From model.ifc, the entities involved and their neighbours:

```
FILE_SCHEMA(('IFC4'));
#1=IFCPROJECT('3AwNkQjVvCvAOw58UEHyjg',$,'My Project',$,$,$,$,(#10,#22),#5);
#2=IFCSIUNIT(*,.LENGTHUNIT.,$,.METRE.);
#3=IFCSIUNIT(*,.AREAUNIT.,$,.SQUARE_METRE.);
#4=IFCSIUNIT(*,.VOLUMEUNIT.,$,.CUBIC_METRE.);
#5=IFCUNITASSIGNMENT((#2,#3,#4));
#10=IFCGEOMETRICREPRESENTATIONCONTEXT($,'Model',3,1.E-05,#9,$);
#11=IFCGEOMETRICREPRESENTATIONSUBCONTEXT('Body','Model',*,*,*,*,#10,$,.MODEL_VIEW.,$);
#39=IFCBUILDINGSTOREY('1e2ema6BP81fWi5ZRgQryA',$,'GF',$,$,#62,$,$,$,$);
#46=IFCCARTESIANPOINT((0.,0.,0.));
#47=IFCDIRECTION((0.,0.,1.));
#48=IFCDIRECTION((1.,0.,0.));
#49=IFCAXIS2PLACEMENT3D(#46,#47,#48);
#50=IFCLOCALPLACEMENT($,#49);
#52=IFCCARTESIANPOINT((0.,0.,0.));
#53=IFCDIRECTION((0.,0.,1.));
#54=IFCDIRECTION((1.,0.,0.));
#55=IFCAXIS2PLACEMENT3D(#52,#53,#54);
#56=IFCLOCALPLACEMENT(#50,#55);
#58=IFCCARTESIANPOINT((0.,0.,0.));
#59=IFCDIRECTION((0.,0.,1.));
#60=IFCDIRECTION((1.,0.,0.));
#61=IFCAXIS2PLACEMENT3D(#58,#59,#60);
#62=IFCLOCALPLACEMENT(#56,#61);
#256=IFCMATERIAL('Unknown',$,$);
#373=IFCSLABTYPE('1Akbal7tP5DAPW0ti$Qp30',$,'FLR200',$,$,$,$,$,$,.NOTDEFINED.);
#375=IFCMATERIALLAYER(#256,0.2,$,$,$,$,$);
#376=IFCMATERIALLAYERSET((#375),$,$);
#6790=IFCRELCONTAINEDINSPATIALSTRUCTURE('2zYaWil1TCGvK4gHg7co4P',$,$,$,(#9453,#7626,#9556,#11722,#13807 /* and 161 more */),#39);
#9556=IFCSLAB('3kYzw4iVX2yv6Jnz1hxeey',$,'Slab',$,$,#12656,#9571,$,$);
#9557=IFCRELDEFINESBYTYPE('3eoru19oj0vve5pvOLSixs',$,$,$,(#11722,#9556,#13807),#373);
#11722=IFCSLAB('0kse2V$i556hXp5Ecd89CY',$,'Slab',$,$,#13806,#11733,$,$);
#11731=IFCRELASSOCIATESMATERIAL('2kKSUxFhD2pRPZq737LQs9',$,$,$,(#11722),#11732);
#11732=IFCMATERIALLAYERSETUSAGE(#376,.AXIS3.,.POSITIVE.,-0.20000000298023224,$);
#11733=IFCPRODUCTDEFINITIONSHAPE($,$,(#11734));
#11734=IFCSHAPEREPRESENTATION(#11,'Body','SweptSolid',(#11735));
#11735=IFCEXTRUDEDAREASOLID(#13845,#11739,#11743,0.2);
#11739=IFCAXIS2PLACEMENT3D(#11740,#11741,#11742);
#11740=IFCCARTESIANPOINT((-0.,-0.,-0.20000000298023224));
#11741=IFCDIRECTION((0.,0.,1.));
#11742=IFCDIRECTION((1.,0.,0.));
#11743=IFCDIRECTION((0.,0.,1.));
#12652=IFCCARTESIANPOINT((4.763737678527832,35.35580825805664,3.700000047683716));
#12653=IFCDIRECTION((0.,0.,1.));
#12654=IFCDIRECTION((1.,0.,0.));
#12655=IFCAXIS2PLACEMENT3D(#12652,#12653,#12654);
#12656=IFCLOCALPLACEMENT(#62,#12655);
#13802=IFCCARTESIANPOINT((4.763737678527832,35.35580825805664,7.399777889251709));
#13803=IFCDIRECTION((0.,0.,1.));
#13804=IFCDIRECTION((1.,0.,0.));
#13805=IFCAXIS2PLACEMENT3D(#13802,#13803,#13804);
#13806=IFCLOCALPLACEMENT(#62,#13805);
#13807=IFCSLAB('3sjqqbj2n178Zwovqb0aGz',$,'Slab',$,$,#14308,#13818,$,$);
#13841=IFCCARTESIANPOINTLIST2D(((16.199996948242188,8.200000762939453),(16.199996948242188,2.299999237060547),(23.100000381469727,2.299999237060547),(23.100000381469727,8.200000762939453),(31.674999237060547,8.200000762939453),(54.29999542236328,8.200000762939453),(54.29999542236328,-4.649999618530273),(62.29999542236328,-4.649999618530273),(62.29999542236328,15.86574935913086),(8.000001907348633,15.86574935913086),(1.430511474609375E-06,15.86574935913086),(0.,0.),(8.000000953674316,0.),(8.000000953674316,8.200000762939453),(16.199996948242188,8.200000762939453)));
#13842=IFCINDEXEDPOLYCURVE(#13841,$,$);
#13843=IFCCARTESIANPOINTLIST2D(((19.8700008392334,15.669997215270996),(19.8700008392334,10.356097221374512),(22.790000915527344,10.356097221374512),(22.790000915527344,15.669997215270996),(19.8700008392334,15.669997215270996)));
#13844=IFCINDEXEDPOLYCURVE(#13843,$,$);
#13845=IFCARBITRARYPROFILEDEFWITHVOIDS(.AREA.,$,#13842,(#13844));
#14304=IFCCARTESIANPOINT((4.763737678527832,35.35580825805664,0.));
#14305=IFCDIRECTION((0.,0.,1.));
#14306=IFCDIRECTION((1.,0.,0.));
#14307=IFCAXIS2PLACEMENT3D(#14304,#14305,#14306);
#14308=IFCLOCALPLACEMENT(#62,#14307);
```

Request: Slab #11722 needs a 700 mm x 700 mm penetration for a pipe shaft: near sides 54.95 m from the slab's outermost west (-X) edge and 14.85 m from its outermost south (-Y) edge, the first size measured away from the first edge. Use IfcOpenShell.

```python
import numpy as np
import ifcopenshell
import ifcopenshell.api.feature
import ifcopenshell.api.geometry
import ifcopenshell.api.root
import ifcopenshell.geom
import ifcopenshell.util.placement
import ifcopenshell.util.representation
import ifcopenshell.util.shape
import ifcopenshell.util.unit

model = ifcopenshell.open("model.ifc")
unit_scale = ifcopenshell.util.unit.calculate_unit_scale(model)
settings = ifcopenshell.geom.settings()


def volume(element):
    """Net volume in cubic metres, openings subtracted."""
    shape = ifcopenshell.geom.create_shape(settings, element)
    return ifcopenshell.util.shape.get_volume(shape.geometry)


slab = model.by_guid("0kse2V$i556hXp5Ecd89CY")
before = volume(slab)

# Extent in the slab's own axes, in metres. The edges named are its -X and -Y sides.
slab_shape = ifcopenshell.geom.create_shape(settings, slab)
vertices = ifcopenshell.util.shape.get_vertices(slab_shape.geometry)
x_min, y_min, bottom = vertices.min(axis=0)
top = vertices[:, 2].max()

opening = ifcopenshell.api.root.create_entity(model, ifc_class="IfcOpeningElement", name="Pipe shaft opening", predefined_type="OPENING")
context = ifcopenshell.util.representation.get_context(model, "Model", "Body", "MODEL_VIEW")
width, depth = 0.7, 0.7
outline = [(0.0, 0.0), (width, 0.0), (width, depth), (0.0, depth), (0.0, 0.0)]
# Overshoot both faces by 50 mm so the cut is clean.
shape = ifcopenshell.api.geometry.add_slab_representation(
    model, context=context, depth=top - bottom + 0.1, polyline=outline
)
ifcopenshell.api.geometry.assign_representation(model, product=opening, representation=shape)

matrix = ifcopenshell.util.placement.get_local_placement(slab.ObjectPlacement)
matrix[:, 3] = matrix @ np.append(np.array([x_min + 54.95, y_min + 14.85, bottom - 0.05]) / unit_scale, 1.0)
ifcopenshell.api.geometry.edit_object_placement(model, product=opening, matrix=matrix, is_si=False)
ifcopenshell.api.feature.add_feature(model, feature=opening, element=slab)

after = volume(slab)

print(f"slab volume {before:.3f} -> {after:.3f} m3")

model.write("model_rev.ifc")
```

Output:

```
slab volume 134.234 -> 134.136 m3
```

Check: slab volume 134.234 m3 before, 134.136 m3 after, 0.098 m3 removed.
